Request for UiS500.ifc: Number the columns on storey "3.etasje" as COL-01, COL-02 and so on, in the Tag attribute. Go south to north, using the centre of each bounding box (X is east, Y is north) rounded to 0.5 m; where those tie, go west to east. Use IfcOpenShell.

First a look at what the model holds.

```python
import ifcopenshell
import ifcopenshell.util.element
import ifcopenshell.util.placement

model = ifcopenshell.open("UiS500.ifc")
print(model.schema)
storey = next(s for s in model.by_type("IfcBuildingStorey") if s.Name == "3.etasje")
columns = [e for e in ifcopenshell.util.element.get_decomposition(storey) if e.is_a("IfcColumn")]
for e in sorted(columns, key=lambda e: e.id()):
    origin = ifcopenshell.util.placement.get_local_placement(e.ObjectPlacement)[:3, 3]
    print(e.id(), e.Tag, e.Name, origin.round(2) + 0.0, sep=" | ")
```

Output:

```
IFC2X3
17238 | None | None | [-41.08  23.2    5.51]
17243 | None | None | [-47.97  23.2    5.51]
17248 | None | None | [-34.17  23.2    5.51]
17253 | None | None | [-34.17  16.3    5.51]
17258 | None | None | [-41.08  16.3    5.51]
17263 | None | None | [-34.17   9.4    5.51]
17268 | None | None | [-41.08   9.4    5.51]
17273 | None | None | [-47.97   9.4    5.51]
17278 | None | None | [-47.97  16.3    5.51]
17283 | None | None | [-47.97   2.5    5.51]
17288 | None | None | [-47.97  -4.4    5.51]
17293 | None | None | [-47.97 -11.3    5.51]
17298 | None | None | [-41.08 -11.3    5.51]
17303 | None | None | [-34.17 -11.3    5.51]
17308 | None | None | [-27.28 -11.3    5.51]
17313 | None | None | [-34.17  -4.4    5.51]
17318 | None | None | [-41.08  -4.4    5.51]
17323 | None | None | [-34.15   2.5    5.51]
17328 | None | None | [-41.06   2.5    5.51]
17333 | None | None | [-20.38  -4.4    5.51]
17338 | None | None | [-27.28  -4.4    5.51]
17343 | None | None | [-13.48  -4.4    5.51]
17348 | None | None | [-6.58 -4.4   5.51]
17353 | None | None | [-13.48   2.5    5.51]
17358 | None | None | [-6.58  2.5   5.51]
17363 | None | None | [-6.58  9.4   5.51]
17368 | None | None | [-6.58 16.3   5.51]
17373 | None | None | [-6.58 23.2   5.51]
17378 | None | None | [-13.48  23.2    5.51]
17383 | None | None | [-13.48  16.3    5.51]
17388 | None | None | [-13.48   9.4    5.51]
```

```python
import ifcopenshell
import ifcopenshell.geom
import ifcopenshell.util.element
import ifcopenshell.util.shape

model = ifcopenshell.open("UiS500.ifc")
settings = ifcopenshell.geom.settings()
settings.set("use-world-coords", True)


def centre(element):
    shape = ifcopenshell.geom.create_shape(settings, element)
    return ifcopenshell.util.shape.get_bbox_centroid(shape.geometry)


storey = next(s for s in model.by_type("IfcBuildingStorey") if s.Name == "3.etasje")
columns = [e for e in ifcopenshell.util.element.get_decomposition(storey) if e.is_a("IfcColumn")]

# Insertion points can sit at a corner or the storey origin, so sort by the geometry (in metres).
centres = {e: centre(e) for e in columns}
columns.sort(key=lambda e: (round(centres[e][1] / 0.5), centres[e][0]))

for i, e in enumerate(columns, start=1):
    number = f"COL-{i:02d}"
    e.Tag = number
    print(e.id(), number)

model.write("UiS500_rev.ifc")
```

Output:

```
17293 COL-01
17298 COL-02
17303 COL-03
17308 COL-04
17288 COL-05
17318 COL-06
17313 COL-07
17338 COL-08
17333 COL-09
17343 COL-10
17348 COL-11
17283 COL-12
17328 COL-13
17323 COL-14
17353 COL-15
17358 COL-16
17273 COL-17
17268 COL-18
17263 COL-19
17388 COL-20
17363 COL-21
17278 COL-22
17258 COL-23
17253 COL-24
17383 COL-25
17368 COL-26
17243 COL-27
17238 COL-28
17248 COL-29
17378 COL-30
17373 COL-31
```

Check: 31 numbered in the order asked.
